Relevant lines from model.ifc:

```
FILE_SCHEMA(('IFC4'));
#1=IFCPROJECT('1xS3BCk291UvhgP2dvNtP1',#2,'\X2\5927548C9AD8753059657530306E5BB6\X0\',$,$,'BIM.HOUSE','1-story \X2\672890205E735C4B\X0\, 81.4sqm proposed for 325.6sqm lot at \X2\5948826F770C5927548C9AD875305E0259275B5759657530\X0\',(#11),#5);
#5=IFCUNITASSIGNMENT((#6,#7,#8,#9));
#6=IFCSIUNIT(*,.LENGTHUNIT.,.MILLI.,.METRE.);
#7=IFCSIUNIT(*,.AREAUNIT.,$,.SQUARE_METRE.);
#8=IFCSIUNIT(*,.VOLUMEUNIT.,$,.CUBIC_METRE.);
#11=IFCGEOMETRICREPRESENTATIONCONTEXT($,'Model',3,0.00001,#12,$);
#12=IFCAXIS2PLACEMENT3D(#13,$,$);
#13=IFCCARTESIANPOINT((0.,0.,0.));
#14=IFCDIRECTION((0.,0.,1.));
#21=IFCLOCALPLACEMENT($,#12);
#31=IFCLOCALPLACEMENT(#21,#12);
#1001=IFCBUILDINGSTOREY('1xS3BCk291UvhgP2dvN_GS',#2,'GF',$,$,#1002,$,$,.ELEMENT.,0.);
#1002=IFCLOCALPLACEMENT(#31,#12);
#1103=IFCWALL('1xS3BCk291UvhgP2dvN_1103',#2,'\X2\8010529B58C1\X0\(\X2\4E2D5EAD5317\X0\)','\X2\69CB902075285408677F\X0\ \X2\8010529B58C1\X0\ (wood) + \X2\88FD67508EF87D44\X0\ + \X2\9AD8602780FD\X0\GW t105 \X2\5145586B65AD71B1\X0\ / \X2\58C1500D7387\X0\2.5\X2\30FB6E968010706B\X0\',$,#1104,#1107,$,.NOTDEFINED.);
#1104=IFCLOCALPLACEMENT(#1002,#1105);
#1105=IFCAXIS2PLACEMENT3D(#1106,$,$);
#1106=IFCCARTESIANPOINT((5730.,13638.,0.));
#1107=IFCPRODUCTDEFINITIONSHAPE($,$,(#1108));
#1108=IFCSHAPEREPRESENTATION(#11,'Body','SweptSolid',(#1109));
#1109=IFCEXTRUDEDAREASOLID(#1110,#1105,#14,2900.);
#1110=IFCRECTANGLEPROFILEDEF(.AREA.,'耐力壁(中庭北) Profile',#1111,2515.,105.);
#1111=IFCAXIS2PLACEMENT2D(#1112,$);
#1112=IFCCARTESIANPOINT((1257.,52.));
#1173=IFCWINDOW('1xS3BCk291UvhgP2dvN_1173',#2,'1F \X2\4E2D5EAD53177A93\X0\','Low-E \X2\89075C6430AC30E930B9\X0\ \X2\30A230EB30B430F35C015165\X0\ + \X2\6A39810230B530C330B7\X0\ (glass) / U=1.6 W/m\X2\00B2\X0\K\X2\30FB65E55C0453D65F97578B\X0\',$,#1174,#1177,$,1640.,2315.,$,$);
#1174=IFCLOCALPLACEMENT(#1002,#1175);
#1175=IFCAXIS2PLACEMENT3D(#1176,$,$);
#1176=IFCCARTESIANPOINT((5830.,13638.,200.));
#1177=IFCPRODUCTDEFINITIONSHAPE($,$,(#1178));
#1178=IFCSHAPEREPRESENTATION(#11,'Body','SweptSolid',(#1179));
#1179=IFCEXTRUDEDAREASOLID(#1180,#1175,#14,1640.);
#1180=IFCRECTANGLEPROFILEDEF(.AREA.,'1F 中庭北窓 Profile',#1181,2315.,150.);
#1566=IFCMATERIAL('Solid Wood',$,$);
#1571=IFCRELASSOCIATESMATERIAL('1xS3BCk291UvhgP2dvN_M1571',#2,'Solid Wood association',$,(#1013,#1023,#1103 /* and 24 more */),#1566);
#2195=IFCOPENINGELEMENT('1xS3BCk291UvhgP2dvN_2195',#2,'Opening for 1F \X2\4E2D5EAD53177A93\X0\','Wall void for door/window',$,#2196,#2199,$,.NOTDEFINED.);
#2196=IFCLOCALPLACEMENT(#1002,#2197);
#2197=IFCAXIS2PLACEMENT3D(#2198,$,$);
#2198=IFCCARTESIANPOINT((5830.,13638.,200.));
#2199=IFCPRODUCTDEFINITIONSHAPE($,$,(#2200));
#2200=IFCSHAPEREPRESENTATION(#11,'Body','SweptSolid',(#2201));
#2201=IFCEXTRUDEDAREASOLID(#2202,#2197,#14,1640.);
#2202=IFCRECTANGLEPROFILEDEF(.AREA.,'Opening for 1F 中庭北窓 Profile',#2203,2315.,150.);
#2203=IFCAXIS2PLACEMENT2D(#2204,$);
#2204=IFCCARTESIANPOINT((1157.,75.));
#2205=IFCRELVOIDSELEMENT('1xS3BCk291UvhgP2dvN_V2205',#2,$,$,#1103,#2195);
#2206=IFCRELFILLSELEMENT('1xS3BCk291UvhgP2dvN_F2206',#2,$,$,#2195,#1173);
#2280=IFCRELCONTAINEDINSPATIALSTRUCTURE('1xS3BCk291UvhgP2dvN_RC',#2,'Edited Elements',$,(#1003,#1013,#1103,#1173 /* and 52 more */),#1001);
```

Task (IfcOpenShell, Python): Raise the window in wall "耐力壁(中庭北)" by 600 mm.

```python
import numpy as np
import ifcopenshell
import ifcopenshell.api.geometry
import ifcopenshell.util.placement
import ifcopenshell.util.unit

model = ifcopenshell.open("model.ifc")
unit_scale = ifcopenshell.util.unit.calculate_unit_scale(model)

window = model.by_id(1173)
opening = window.FillsVoids[0].RelatingOpeningElement
dz = 600.0

shift = np.array([0.0, 0.0, dz])
# The window is not placed relative to its opening, so move both.
for product in (opening, window):
    matrix = ifcopenshell.util.placement.get_local_placement(product.ObjectPlacement)
    matrix[:3, 3] += shift
    ifcopenshell.api.geometry.edit_object_placement(model, product=product, matrix=matrix, is_si=False)

print(f"moved by {dz * unit_scale:+.3f} m")

model.write("model_rev.ifc")
```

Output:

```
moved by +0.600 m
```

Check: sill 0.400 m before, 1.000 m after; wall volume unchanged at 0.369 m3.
